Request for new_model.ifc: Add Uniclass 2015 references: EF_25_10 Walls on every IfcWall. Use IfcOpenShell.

First a look at what the model holds.

```python
import ifcopenshell

model = ifcopenshell.open("new_model.ifc")
print(model.schema)
print("classifications:", [c.Name for c in model.by_type("IfcClassification")])
for ifc_class in ("IfcDoor", "IfcRoof", "IfcStair", "IfcWall", "IfcWindow"):
    print(ifc_class, len(model.by_type(ifc_class)))
```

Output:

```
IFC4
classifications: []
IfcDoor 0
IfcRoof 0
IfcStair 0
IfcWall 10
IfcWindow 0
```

```python
import ifcopenshell
import ifcopenshell.api.classification

model = ifcopenshell.open("new_model.ifc")

system = ifcopenshell.api.classification.add_classification(model, classification="Uniclass 2015")

codes = {
    "IfcWall": ("EF_25_10", "Walls"),
}
for ifc_class, (code, name) in codes.items():
    products = model.by_type(ifc_class)
    ifcopenshell.api.classification.add_reference(
        model, products=products, classification=system, identification=code, name=name
    )
    print(code, len(products))

model.write("new_model_edited.ifc")
```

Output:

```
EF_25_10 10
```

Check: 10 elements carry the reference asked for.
